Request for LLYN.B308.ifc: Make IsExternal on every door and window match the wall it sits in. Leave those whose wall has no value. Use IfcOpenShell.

First a look at what the model holds.

```python
import ifcopenshell
import ifcopenshell.util.element

model = ifcopenshell.open("LLYN.B308.ifc")
print(model.schema)
seen = {}
for e in model.by_type("IfcDoor") + model.by_type("IfcWindow"):
    if not e.FillsVoids:
        continue
    host = e.FillsVoids[0].RelatingOpeningElement.VoidsElements[0].RelatingBuildingElement
    own = ifcopenshell.util.element.get_pset(e, f"Pset_{e.is_a()[3:].removesuffix('StandardCase')}Common", "IsExternal")
    wall = ifcopenshell.util.element.get_pset(host, "Pset_WallCommon", "IsExternal")
    seen[e.is_a(), own, wall] = seen.get((e.is_a(), own, wall), 0) + 1
for (cls, own, wall), count in sorted(seen.items(), key=str):
    print(count, cls, "IsExternal:", own, "| host wall:", wall)
```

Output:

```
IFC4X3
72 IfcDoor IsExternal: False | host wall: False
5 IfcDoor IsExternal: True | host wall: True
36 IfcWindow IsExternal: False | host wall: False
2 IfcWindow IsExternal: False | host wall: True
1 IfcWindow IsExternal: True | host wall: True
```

```python
import ifcopenshell
import ifcopenshell.api.pset
import ifcopenshell.util.element

model = ifcopenshell.open("LLYN.B308.ifc")

count = 0
for ifc_class, pset_name in (("IfcDoor", "Pset_DoorCommon"), ("IfcWindow", "Pset_WindowCommon")):
    for e in model.by_type(ifc_class):
        if not e.FillsVoids:
            continue
        host = e.FillsVoids[0].RelatingOpeningElement.VoidsElements[0].RelatingBuildingElement
        external = ifcopenshell.util.element.get_pset(host, "Pset_WallCommon", "IsExternal")
        if external is None or ifcopenshell.util.element.get_pset(e, pset_name, "IsExternal") == external:
            continue
        pset = ifcopenshell.api.pset.add_pset(model, product=e, name=pset_name)
        ifcopenshell.api.pset.edit_pset(model, pset=pset, properties={"IsExternal": external})
        count += 1

print(count, "updated")

model.write("LLYN.B308-out.ifc")
```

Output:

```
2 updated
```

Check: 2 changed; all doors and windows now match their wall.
